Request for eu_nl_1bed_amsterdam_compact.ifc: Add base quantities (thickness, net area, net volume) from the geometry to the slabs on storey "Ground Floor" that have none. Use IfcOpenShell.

First a look at what the model holds.

```python
import ifcopenshell
import ifcopenshell.util.element
import ifcopenshell.util.unit

model = ifcopenshell.open("eu_nl_1bed_amsterdam_compact.ifc")
print(model.schema)
for unit_type in ("LENGTHUNIT", "AREAUNIT", "VOLUMEUNIT"):
    print(unit_type, ifcopenshell.util.unit.calculate_unit_scale(model, unit_type))
storey = next(s for s in model.by_type("IfcBuildingStorey") if s.Name == "Ground Floor")
slabs = [e for e in ifcopenshell.util.element.get_decomposition(storey) if e.is_a("IfcSlab")]
for e in sorted(slabs, key=lambda e: e.id()):
    print(e.id(), e.is_a(), e.Name, list(ifcopenshell.util.element.get_psets(e, qtos_only=True)), sep=" | ")
```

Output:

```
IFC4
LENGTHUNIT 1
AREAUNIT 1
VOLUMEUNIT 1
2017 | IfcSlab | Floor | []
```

```python
import ifcopenshell
import ifcopenshell.api.pset
import ifcopenshell.geom
import ifcopenshell.util.element
import ifcopenshell.util.shape
import ifcopenshell.util.unit

model = ifcopenshell.open("eu_nl_1bed_amsterdam_compact.ifc")
unit_scale = ifcopenshell.util.unit.calculate_unit_scale(model)
area_scale = ifcopenshell.util.unit.calculate_unit_scale(model, "AREAUNIT")
volume_scale = ifcopenshell.util.unit.calculate_unit_scale(model, "VOLUMEUNIT")
settings = ifcopenshell.geom.settings()

storey = next(s for s in model.by_type("IfcBuildingStorey") if s.Name == "Ground Floor")
slabs = [e for e in ifcopenshell.util.element.get_decomposition(storey) if e.is_a("IfcSlab")]

for e in sorted(slabs, key=lambda e: e.id()):
    if ifcopenshell.util.element.get_psets(e, qtos_only=True, should_inherit=False):
        continue
    # Geometry comes back in metres, in the element's own axes.
    shape = ifcopenshell.geom.create_shape(settings, e)
    values = {
        "Width": ifcopenshell.util.shape.get_z(shape.geometry) / unit_scale,
        "NetArea": ifcopenshell.util.shape.get_footprint_area(shape.geometry) / area_scale,
        "NetVolume": ifcopenshell.util.shape.get_volume(shape.geometry) / volume_scale,
    }
    qto = ifcopenshell.api.pset.add_qto(model, product=e, name="Qto_SlabBaseQuantities")
    ifcopenshell.api.pset.edit_qto(model, qto=qto, properties=values)
    print(e.id(), {k: round(v, 3) for k, v in values.items()})

model.write("eu_nl_1bed_amsterdam_compact_edited.ifc")
```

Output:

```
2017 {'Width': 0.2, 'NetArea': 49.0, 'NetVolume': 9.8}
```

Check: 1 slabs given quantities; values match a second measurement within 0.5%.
